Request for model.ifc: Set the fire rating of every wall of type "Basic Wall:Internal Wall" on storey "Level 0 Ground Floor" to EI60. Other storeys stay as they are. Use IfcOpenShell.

First a look at what the model holds.

```python
import ifcopenshell
import ifcopenshell.util.element

model = ifcopenshell.open("model.ifc")
print(model.schema)
storey = next(s for s in model.by_type("IfcBuildingStorey") if s.Name == "Level 0 Ground Floor")
walls = [e for e in ifcopenshell.util.element.get_decomposition(storey) if e.is_a("IfcWall")]
seen = {}
for e in walls:
    element_type = ifcopenshell.util.element.get_type(e)
    key = (element_type.Name if element_type != e and element_type else None, ifcopenshell.util.element.get_pset(e, "Pset_WallCommon", "FireRating"))
    seen[key] = seen.get(key, 0) + 1
for (name, value), count in sorted(seen.items(), key=str):
    print(count, "x", name, "|", value)
```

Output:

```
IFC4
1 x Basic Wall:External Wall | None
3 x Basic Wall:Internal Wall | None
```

```python
import ifcopenshell
import ifcopenshell.api.pset
import ifcopenshell.util.element

model = ifcopenshell.open("model.ifc")

storey = next(s for s in model.by_type("IfcBuildingStorey") if s.Name == "Level 0 Ground Floor")
walls = [e for e in ifcopenshell.util.element.get_decomposition(storey) if e.is_a("IfcWall")]

count = 0
for e in walls:
    element_type = ifcopenshell.util.element.get_type(e)
    if element_type in (None, e) or element_type.Name != "Basic Wall:Internal Wall":
        continue
    # add_pset returns the element's existing set when there is one.
    pset = ifcopenshell.api.pset.add_pset(model, product=e, name="Pset_WallCommon")
    ifcopenshell.api.pset.edit_pset(model, pset=pset, properties={"FireRating": "EI60"})
    count += 1

print(count, "walls updated")

model.write("model_updated.ifc")
```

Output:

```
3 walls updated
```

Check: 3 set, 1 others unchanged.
